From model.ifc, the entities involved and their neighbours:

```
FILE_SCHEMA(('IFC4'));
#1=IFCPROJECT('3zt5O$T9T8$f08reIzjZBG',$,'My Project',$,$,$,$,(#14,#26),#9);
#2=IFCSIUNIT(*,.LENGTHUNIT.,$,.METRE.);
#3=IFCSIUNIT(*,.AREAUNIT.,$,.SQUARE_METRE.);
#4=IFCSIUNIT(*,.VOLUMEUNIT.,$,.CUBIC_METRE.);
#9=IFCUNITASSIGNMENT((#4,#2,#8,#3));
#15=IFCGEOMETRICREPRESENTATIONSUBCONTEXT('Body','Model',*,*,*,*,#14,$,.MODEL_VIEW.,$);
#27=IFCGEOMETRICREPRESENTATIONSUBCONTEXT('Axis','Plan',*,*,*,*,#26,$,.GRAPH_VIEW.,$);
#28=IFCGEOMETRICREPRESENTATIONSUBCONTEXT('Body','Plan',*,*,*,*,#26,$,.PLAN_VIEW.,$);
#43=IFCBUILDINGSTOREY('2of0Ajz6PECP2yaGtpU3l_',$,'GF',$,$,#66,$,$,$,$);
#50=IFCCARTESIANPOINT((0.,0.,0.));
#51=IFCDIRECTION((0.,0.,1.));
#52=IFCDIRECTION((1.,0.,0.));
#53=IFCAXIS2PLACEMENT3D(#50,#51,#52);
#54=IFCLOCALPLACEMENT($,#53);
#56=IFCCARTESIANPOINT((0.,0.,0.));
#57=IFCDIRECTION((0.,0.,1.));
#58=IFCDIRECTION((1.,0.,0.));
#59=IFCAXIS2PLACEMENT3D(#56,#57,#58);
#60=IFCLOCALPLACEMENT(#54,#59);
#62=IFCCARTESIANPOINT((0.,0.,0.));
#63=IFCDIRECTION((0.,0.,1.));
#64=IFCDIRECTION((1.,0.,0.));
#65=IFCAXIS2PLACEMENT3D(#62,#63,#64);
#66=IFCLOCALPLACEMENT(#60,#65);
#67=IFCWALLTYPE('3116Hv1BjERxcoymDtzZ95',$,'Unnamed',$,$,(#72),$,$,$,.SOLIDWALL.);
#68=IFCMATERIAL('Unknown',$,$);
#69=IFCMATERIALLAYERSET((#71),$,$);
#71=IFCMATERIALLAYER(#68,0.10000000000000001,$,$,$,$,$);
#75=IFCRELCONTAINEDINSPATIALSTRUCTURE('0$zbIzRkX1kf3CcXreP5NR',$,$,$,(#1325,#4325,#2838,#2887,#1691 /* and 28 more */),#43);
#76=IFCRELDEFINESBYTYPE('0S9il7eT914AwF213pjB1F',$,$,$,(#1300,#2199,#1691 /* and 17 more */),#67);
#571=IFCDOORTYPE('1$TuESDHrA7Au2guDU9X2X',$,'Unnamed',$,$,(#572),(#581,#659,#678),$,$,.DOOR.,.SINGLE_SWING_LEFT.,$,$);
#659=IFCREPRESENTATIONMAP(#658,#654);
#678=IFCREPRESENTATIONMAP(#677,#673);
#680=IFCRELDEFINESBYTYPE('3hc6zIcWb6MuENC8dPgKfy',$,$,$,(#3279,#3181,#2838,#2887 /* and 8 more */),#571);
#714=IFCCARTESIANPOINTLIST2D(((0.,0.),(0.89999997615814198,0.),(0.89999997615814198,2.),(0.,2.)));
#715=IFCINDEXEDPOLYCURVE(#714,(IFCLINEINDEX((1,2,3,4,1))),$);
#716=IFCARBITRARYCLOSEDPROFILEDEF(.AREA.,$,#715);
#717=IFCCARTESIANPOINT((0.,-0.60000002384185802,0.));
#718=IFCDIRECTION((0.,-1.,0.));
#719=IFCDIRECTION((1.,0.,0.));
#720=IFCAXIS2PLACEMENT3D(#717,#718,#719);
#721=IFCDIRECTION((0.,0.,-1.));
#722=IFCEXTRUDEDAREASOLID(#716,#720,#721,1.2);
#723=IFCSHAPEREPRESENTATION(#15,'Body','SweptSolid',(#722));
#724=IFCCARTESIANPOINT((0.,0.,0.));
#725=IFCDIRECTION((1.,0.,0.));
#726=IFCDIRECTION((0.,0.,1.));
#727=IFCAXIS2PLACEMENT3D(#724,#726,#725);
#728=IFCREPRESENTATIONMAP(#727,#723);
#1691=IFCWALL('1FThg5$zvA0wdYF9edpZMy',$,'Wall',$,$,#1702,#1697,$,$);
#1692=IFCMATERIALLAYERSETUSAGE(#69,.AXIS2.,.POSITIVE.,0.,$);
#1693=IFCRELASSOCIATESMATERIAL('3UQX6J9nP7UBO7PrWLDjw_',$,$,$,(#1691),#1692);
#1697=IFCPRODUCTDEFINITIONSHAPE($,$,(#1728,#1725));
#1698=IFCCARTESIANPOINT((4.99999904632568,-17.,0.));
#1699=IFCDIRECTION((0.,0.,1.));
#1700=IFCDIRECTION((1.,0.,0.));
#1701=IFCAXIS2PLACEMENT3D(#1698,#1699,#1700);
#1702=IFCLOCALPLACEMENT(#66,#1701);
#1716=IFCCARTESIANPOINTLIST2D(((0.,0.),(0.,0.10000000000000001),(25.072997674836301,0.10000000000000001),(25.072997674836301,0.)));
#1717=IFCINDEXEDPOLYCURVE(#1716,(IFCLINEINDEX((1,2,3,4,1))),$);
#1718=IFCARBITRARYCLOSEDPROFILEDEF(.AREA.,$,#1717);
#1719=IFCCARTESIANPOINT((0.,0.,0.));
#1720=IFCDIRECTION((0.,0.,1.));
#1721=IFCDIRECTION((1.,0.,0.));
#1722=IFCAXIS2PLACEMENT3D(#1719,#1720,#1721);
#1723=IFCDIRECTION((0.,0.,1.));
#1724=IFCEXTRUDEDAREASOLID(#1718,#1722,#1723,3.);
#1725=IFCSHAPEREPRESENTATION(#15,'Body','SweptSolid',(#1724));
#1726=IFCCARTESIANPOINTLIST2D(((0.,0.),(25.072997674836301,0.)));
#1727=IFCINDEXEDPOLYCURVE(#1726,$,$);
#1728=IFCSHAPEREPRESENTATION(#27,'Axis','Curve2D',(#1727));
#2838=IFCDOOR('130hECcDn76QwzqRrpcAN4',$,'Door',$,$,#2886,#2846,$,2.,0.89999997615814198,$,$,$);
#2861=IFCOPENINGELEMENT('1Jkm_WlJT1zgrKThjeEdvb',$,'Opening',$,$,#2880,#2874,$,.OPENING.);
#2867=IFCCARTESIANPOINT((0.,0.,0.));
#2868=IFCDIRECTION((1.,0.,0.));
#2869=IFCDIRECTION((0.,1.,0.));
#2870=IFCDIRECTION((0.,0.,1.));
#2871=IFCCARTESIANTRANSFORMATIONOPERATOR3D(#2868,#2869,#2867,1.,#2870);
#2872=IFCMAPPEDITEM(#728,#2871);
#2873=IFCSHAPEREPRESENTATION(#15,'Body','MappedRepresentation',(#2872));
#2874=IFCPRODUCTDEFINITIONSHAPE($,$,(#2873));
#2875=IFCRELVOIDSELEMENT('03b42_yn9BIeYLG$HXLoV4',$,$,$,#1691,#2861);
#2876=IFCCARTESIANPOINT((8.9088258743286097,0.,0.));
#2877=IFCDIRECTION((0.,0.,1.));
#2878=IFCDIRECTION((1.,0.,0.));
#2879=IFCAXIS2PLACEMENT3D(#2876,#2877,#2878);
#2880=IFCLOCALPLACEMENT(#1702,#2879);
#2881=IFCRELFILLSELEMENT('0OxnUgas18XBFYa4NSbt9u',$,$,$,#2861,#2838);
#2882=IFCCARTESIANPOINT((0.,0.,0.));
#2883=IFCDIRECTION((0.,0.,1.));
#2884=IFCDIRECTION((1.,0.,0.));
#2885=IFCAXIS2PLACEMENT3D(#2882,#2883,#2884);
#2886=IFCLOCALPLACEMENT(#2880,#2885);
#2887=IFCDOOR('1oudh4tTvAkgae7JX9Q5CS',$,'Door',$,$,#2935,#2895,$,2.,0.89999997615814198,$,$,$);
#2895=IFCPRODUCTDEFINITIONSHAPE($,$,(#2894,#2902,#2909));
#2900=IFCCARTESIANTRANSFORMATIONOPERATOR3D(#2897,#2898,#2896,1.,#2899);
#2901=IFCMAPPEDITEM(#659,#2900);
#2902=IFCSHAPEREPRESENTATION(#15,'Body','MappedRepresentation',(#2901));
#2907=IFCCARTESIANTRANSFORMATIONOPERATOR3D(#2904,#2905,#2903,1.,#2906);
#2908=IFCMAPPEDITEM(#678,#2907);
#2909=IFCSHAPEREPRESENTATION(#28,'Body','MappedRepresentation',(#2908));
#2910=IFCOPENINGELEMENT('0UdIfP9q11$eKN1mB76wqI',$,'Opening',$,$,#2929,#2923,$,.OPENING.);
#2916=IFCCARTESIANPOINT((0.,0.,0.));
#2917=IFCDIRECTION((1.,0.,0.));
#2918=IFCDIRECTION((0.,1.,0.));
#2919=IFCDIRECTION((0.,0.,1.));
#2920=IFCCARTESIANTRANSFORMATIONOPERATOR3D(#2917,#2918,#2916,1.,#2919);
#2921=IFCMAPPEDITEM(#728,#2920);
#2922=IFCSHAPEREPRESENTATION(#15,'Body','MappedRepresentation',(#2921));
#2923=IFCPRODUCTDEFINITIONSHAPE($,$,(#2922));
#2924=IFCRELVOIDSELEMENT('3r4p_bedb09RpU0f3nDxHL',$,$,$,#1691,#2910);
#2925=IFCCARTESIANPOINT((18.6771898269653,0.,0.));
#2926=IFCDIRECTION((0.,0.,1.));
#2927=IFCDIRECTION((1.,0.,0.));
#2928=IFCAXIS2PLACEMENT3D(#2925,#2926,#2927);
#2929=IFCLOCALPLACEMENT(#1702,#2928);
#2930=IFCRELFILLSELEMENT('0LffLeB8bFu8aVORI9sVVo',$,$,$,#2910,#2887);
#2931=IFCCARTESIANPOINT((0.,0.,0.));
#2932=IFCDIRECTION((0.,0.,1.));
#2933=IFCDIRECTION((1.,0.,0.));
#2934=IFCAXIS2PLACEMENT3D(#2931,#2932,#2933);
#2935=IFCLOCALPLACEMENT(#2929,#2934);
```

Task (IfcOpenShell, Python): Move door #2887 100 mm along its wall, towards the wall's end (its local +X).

```python
import ifcopenshell
import ifcopenshell.api.geometry
import ifcopenshell.util.placement

model = ifcopenshell.open("model.ifc")

door = model.by_guid("1oudh4tTvAkgae7JX9Q5CS")
opening = door.FillsVoids[0].RelatingOpeningElement
wall = opening.VoidsElements[0].RelatingBuildingElement

wall_matrix = ifcopenshell.util.placement.get_local_placement(wall.ObjectPlacement)
shift = wall_matrix[:3, 0] * 0.1
before = ifcopenshell.util.placement.get_local_placement(door.ObjectPlacement)[:3, 3].copy()

# The door is placed relative to its opening, so it follows when the opening moves.
matrix = ifcopenshell.util.placement.get_local_placement(opening.ObjectPlacement)
matrix[:3, 3] += shift
ifcopenshell.api.geometry.edit_object_placement(
    model, product=opening, matrix=matrix, is_si=False, should_transform_children=True
)

after = ifcopenshell.util.placement.get_local_placement(door.ObjectPlacement)[:3, 3]
print("door moved by", (after - before).round(3) + 0.0)

model.write("model_rev.ifc")
```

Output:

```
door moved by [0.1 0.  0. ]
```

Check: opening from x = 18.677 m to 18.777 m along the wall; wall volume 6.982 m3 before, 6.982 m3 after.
